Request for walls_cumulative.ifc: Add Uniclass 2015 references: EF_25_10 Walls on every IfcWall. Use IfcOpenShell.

First a look at what the model holds.

```python
import ifcopenshell

model = ifcopenshell.open("walls_cumulative.ifc")
print(model.schema)
print("classifications:", [c.Name for c in model.by_type("IfcClassification")])
for ifc_class in ("IfcDoor", "IfcRoof", "IfcStair", "IfcWall", "IfcWindow"):
    print(ifc_class, len(model.by_type(ifc_class)))
```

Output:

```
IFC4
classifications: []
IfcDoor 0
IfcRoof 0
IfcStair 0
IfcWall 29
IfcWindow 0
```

```python
import ifcopenshell
import ifcopenshell.api.classification

model = ifcopenshell.open("walls_cumulative.ifc")

system = ifcopenshell.api.classification.add_classification(model, classification="Uniclass 2015")

codes = {
    "IfcWall": ("EF_25_10", "Walls"),
}
for ifc_class, (code, name) in codes.items():
    products = model.by_type(ifc_class)
    ifcopenshell.api.classification.add_reference(
        model, products=products, classification=system, identification=code, name=name
    )
    print(code, len(products))

model.write("walls_cumulative_v2.ifc")
```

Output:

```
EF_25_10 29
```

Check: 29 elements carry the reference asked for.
